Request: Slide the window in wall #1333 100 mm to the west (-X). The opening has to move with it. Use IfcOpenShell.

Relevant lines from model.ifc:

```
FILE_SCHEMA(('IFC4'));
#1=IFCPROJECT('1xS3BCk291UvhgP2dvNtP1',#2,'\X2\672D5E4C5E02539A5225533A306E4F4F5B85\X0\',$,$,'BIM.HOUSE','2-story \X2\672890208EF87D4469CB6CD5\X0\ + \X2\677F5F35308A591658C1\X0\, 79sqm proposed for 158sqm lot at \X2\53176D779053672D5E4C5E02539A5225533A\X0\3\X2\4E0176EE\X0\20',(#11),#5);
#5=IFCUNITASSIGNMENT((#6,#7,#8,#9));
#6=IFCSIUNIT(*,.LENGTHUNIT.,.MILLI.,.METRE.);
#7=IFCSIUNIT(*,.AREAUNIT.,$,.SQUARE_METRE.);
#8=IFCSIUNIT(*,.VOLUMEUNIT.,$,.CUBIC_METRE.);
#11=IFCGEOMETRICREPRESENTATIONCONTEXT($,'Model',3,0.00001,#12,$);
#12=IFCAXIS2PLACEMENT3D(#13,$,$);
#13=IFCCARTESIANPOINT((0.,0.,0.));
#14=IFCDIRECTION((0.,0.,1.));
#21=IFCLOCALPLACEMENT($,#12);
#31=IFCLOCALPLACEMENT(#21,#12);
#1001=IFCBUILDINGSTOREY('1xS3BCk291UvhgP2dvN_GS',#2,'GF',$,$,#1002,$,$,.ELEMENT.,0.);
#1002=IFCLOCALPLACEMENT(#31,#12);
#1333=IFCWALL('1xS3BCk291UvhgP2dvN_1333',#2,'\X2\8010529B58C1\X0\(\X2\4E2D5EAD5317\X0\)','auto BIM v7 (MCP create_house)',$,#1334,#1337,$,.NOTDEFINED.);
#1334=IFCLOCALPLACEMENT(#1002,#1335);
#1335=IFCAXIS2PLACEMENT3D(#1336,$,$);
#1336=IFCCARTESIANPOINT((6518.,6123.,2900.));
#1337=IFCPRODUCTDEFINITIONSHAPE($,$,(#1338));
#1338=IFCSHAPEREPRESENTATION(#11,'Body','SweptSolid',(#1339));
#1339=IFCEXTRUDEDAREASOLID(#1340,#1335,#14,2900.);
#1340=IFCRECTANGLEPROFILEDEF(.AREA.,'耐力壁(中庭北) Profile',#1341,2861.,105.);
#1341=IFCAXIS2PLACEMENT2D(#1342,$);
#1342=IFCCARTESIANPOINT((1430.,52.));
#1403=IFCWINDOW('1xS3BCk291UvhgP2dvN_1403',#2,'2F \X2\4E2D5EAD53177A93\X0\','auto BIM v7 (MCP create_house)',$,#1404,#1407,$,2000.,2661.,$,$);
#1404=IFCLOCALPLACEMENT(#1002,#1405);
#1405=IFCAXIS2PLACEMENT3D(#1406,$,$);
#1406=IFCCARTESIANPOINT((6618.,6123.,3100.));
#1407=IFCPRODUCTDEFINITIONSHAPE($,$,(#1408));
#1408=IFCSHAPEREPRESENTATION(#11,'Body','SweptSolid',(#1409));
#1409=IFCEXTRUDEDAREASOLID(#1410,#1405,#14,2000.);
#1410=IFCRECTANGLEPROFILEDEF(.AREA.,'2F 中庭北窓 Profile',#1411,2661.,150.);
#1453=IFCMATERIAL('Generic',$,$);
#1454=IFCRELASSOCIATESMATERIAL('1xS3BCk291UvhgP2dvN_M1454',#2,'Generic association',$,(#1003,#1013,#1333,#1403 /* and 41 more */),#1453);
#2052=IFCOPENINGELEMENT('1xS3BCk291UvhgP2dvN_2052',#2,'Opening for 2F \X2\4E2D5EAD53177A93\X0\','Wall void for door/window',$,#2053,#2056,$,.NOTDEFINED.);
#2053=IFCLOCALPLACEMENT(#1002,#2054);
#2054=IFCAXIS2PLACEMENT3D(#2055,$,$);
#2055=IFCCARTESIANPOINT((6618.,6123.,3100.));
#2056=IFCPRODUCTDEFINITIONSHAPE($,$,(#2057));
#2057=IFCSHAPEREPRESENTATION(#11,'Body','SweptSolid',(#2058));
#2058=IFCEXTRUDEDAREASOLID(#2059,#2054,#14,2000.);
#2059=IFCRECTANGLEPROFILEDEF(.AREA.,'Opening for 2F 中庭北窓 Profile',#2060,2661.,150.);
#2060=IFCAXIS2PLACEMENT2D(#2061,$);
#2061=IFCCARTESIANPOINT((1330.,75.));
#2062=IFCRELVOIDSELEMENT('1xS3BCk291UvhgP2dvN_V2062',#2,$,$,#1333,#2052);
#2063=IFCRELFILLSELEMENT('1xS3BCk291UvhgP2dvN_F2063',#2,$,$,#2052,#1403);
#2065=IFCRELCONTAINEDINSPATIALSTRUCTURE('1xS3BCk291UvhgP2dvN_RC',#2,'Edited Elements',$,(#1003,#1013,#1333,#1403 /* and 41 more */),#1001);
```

```python
import ifcopenshell
import ifcopenshell.api.geometry
import ifcopenshell.util.placement

model = ifcopenshell.open("model.ifc")

window = model.by_id(1403)
opening = window.FillsVoids[0].RelatingOpeningElement
wall = opening.VoidsElements[0].RelatingBuildingElement

wall_matrix = ifcopenshell.util.placement.get_local_placement(wall.ObjectPlacement)
shift = wall_matrix[:3, 0] * -100.0
before = ifcopenshell.util.placement.get_local_placement(window.ObjectPlacement)[:3, 3].copy()

# The window is not placed relative to its opening, so move both.
for product in (opening, window):
    matrix = ifcopenshell.util.placement.get_local_placement(product.ObjectPlacement)
    matrix[:3, 3] += shift
    ifcopenshell.api.geometry.edit_object_placement(model, product=product, matrix=matrix, is_si=False)

after = ifcopenshell.util.placement.get_local_placement(window.ObjectPlacement)[:3, 3]
print("window moved by", (after - before).round(3) + 0.0)

model.write("model_rev.ifc")
```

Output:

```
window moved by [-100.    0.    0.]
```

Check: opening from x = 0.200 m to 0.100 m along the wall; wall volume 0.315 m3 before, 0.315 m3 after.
